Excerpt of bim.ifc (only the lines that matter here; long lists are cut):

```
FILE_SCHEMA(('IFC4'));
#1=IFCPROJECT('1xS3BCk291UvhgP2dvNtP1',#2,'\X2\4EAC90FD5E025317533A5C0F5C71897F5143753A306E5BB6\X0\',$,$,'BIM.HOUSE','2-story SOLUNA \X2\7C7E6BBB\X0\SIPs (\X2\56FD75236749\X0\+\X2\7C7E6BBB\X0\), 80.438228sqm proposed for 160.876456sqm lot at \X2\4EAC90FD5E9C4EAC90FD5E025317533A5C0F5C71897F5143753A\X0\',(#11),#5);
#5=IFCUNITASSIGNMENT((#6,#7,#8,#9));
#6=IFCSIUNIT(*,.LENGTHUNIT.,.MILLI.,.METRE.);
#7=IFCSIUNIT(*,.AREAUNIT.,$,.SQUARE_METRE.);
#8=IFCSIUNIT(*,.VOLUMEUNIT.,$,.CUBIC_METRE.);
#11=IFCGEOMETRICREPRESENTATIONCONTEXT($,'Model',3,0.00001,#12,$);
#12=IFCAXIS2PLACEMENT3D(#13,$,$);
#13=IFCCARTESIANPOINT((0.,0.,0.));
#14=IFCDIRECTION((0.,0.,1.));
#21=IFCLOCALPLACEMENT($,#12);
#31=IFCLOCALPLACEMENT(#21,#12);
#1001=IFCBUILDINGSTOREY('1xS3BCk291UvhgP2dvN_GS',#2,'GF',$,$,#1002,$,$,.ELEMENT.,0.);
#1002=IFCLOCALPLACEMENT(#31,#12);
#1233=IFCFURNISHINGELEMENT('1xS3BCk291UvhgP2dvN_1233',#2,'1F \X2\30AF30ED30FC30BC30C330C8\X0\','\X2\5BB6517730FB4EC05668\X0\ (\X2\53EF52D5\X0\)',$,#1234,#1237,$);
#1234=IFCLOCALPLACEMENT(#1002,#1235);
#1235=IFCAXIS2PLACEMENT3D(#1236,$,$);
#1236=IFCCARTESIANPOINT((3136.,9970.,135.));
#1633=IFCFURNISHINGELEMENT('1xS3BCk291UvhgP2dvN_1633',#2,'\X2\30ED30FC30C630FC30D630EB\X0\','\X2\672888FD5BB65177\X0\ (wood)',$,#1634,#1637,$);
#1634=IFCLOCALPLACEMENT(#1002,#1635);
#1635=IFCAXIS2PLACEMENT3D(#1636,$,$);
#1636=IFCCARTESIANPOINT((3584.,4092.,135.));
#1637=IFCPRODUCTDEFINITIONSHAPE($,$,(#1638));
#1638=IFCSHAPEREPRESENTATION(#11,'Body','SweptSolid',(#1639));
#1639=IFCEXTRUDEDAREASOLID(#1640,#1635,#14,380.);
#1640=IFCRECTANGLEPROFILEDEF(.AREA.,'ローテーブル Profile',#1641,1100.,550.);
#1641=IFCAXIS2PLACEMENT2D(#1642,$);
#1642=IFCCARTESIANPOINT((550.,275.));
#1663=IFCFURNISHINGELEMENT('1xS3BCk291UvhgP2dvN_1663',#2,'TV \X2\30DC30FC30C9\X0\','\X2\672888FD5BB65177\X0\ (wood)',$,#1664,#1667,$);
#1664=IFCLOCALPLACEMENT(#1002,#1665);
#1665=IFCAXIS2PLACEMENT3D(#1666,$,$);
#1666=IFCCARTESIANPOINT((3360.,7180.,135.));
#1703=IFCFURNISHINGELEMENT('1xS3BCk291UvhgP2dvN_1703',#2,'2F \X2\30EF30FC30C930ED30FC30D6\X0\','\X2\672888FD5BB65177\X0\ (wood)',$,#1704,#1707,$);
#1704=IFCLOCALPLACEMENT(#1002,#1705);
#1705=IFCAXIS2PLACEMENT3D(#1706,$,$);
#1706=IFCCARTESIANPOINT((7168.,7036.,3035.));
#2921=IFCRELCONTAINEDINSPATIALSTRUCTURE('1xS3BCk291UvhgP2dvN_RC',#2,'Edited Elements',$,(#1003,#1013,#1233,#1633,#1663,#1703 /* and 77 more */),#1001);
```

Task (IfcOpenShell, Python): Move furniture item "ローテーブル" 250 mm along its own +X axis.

```python
import ifcopenshell
import ifcopenshell.api.geometry
import ifcopenshell.util.placement
import ifcopenshell.util.unit

model = ifcopenshell.open("bim.ifc")
unit_scale = ifcopenshell.util.unit.calculate_unit_scale(model)

item = model.by_guid("1xS3BCk291UvhgP2dvN_1633")
matrix = ifcopenshell.util.placement.get_local_placement(item.ObjectPlacement)
matrix[:3, 3] += matrix[:3, 0] * 0.25 / unit_scale
ifcopenshell.api.geometry.edit_object_placement(model, product=item, matrix=matrix, is_si=False)

print(ifcopenshell.util.placement.get_local_placement(item.ObjectPlacement).round(3) + 0.0)

model.write("bim_rev.ifc")
```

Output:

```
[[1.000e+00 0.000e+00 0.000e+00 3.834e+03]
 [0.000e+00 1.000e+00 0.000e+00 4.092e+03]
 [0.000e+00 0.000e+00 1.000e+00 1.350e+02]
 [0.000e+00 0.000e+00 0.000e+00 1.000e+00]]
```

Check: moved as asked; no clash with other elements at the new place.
